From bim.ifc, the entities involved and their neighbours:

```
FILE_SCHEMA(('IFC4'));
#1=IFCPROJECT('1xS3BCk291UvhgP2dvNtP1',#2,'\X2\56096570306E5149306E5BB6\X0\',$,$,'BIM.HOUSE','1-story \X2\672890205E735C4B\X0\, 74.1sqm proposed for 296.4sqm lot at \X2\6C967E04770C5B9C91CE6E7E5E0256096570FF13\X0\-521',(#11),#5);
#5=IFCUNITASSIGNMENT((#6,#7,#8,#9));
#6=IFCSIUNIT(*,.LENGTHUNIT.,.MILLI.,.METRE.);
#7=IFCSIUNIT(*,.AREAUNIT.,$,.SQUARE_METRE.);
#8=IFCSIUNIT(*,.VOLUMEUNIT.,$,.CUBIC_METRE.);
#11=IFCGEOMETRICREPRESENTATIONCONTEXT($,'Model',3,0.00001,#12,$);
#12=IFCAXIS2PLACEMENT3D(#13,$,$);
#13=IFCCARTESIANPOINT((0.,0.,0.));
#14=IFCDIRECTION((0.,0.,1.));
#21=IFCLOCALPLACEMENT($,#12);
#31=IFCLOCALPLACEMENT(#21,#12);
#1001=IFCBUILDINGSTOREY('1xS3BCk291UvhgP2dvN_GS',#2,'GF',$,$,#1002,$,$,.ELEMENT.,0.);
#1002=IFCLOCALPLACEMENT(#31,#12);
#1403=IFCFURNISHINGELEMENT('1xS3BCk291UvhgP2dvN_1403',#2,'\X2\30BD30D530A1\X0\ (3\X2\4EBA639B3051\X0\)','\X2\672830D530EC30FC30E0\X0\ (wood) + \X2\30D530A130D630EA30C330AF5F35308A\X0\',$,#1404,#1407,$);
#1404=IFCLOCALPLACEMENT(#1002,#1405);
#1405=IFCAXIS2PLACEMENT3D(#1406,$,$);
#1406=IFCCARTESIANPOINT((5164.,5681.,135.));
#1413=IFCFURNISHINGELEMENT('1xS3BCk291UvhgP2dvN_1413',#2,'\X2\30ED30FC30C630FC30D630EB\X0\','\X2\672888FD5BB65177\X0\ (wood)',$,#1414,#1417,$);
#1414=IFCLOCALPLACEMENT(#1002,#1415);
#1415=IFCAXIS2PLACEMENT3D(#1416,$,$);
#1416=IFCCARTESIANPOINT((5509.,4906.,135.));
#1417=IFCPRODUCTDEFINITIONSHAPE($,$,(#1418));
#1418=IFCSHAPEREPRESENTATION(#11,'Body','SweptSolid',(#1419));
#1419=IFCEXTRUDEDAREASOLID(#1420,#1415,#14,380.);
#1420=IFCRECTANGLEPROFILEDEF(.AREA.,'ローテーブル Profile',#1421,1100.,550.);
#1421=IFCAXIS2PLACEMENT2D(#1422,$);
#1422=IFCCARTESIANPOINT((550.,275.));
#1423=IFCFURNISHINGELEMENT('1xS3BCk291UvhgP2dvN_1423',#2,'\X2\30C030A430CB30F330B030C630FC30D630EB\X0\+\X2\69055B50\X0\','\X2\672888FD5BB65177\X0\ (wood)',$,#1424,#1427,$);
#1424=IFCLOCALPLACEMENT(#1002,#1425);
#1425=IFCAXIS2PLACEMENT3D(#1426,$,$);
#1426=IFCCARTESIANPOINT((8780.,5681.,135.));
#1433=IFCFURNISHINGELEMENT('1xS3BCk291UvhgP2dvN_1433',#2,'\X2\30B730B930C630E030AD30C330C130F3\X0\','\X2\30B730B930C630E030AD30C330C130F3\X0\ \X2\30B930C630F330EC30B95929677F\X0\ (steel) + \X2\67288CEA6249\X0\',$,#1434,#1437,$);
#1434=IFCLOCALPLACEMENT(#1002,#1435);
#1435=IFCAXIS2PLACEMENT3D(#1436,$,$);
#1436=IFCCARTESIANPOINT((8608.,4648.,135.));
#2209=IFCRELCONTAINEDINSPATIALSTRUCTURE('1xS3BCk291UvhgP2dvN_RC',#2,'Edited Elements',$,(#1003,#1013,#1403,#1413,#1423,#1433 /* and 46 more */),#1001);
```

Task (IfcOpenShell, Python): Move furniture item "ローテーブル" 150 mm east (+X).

```python
import ifcopenshell
import ifcopenshell.api.geometry
import ifcopenshell.util.placement
import ifcopenshell.util.unit

model = ifcopenshell.open("bim.ifc")
unit_scale = ifcopenshell.util.unit.calculate_unit_scale(model)

item = model.by_guid("1xS3BCk291UvhgP2dvN_1413")
matrix = ifcopenshell.util.placement.get_local_placement(item.ObjectPlacement)
matrix[0, 3] += 0.15 / unit_scale
ifcopenshell.api.geometry.edit_object_placement(model, product=item, matrix=matrix, is_si=False)

print(ifcopenshell.util.placement.get_local_placement(item.ObjectPlacement).round(3) + 0.0)

model.write("bim_v2.ifc")
```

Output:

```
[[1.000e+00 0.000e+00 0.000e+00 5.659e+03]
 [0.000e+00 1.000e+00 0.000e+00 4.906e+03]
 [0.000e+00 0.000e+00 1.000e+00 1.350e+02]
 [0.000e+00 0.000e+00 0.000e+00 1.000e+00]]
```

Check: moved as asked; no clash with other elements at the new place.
